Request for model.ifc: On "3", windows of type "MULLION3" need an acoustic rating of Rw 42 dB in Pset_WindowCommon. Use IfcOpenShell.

First a look at what the model holds.

```python
import ifcopenshell
import ifcopenshell.util.element

model = ifcopenshell.open("model.ifc")
print(model.schema)
storey = next(s for s in model.by_type("IfcBuildingStorey") if s.Name == "3")
windows = [e for e in ifcopenshell.util.element.get_decomposition(storey) if e.is_a("IfcWindow")]
seen = {}
for e in windows:
    element_type = ifcopenshell.util.element.get_type(e)
    key = (element_type.Name if element_type != e and element_type else None, ifcopenshell.util.element.get_pset(e, "Pset_WindowCommon", "AcousticRating"))
    seen[key] = seen.get(key, 0) + 1
for (name, value), count in sorted(seen.items(), key=str):
    print(count, "x", name, "|", value)
```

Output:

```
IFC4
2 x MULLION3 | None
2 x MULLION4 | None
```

```python
import ifcopenshell
import ifcopenshell.api.pset
import ifcopenshell.util.element

model = ifcopenshell.open("model.ifc")

storey = next(s for s in model.by_type("IfcBuildingStorey") if s.Name == "3")
windows = [e for e in ifcopenshell.util.element.get_decomposition(storey) if e.is_a("IfcWindow")]

count = 0
for e in windows:
    element_type = ifcopenshell.util.element.get_type(e)
    if element_type in (None, e) or element_type.Name != "MULLION3":
        continue
    # add_pset returns the element's existing set when there is one.
    pset = ifcopenshell.api.pset.add_pset(model, product=e, name="Pset_WindowCommon")
    ifcopenshell.api.pset.edit_pset(model, pset=pset, properties={"AcousticRating": "Rw 42 dB"})
    count += 1

print(count, "windows updated")

model.write("model_updated.ifc")
```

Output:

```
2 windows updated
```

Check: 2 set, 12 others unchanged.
